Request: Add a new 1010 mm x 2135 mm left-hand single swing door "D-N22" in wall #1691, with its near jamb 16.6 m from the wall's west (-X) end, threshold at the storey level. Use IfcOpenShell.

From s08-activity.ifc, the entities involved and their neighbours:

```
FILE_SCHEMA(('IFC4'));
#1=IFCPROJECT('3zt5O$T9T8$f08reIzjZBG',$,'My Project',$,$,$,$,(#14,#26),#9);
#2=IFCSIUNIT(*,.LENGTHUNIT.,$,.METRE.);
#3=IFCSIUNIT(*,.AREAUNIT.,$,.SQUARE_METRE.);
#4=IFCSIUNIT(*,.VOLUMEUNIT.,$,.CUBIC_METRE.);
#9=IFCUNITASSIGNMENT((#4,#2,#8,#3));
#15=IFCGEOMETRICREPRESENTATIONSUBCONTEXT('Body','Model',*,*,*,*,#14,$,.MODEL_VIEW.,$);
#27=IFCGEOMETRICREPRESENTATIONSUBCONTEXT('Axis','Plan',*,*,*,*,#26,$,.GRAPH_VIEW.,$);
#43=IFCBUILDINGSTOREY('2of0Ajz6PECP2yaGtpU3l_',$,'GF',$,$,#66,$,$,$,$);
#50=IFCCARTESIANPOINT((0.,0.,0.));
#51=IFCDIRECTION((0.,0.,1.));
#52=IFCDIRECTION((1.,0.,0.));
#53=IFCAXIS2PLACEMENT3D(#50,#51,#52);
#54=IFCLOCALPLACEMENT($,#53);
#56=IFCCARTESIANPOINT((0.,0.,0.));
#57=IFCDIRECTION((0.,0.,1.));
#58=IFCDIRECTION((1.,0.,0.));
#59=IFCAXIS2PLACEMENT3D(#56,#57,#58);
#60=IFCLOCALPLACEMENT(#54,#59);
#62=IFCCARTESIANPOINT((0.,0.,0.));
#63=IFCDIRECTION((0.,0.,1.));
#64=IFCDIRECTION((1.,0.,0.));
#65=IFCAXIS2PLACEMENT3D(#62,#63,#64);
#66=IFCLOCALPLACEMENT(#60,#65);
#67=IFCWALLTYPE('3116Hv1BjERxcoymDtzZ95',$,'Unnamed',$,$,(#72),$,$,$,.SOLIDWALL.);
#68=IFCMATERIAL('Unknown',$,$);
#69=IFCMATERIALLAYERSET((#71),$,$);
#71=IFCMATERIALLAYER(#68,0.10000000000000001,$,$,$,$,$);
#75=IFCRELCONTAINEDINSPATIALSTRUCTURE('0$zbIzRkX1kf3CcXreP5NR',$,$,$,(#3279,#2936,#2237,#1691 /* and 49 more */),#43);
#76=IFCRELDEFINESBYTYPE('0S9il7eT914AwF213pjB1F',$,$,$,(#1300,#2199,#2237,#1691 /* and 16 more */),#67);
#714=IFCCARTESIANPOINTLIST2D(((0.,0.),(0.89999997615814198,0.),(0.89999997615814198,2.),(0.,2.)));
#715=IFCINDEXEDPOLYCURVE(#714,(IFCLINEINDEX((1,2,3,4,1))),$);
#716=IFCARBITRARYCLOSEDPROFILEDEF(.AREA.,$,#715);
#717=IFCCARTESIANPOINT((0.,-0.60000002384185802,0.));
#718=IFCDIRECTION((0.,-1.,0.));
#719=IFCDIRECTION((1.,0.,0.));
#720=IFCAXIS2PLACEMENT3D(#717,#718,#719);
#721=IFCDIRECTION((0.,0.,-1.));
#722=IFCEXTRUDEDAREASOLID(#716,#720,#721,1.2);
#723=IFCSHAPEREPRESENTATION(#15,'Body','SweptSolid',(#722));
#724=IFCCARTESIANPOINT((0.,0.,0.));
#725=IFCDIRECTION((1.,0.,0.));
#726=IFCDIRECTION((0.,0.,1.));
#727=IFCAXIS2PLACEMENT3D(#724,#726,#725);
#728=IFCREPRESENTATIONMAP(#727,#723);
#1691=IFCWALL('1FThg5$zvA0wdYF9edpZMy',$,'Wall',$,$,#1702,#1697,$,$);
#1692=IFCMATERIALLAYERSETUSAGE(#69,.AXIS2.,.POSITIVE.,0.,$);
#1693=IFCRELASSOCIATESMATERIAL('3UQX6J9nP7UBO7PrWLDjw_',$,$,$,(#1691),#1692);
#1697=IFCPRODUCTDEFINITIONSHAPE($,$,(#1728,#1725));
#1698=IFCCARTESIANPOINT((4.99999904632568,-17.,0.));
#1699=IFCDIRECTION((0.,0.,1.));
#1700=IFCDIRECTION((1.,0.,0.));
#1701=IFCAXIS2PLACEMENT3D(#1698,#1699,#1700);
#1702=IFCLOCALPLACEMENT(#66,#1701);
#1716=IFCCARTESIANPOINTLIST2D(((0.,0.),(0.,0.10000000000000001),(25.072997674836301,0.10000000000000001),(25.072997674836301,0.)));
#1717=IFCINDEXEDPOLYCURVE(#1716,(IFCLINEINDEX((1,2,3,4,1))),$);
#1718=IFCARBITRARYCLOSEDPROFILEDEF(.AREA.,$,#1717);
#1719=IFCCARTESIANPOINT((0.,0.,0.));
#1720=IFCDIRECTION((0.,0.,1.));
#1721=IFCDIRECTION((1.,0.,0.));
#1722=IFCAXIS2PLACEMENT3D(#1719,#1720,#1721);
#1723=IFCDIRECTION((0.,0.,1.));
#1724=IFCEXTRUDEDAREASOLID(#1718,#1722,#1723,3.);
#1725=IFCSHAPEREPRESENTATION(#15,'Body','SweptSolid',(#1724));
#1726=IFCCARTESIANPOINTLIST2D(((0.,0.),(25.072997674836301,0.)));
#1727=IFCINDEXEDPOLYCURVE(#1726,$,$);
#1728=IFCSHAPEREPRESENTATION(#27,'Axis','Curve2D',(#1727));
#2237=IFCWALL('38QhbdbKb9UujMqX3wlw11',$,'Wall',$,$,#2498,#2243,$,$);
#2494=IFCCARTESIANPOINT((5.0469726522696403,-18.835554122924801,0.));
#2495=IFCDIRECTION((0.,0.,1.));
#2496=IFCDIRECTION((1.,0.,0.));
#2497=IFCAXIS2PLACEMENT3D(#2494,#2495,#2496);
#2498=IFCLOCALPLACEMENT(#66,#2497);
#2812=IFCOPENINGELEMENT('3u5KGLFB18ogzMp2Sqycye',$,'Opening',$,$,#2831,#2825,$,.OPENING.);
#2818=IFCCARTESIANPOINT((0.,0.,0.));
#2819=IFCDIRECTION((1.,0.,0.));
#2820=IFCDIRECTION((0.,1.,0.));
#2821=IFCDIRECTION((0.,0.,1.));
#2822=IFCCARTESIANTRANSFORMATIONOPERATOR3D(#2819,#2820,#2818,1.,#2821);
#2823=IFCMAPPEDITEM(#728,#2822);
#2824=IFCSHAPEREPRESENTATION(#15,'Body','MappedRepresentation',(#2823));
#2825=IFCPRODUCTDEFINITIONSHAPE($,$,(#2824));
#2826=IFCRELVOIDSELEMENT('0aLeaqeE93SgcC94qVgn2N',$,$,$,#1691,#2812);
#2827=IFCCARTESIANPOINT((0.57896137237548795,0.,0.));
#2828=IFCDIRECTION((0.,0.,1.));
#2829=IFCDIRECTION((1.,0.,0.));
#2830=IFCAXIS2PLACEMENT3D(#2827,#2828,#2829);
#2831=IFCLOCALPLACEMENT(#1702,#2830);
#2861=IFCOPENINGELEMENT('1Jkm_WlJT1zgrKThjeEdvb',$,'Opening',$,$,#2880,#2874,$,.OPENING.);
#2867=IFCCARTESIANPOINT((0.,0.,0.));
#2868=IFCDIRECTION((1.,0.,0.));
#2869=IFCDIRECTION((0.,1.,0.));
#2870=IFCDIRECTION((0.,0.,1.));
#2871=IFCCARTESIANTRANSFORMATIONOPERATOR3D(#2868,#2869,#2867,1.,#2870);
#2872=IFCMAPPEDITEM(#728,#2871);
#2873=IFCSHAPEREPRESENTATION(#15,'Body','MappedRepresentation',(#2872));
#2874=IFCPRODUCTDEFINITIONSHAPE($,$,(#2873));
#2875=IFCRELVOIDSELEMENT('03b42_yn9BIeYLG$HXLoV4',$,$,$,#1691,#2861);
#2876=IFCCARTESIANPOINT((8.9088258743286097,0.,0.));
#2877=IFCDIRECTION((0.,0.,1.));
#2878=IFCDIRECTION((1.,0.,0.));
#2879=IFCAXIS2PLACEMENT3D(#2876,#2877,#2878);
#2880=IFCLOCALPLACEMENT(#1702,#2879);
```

```python
import numpy as np
import ifcopenshell
import ifcopenshell.api.feature
import ifcopenshell.api.geometry
import ifcopenshell.api.root
import ifcopenshell.api.spatial
import ifcopenshell.geom
import ifcopenshell.util.element
import ifcopenshell.util.placement
import ifcopenshell.util.representation
import ifcopenshell.util.shape
import ifcopenshell.util.unit

model = ifcopenshell.open("s08-activity.ifc")
unit_scale = ifcopenshell.util.unit.calculate_unit_scale(model)
settings = ifcopenshell.geom.settings()


def volume(element):
    """Net volume in cubic metres, openings subtracted."""
    shape = ifcopenshell.geom.create_shape(settings, element)
    return ifcopenshell.util.shape.get_volume(shape.geometry)


wall = model.by_guid("1FThg5$zvA0wdYF9edpZMy")
storey = ifcopenshell.util.element.get_container(wall, ifc_class="IfcBuildingStorey")
context = ifcopenshell.util.representation.get_context(model, "Model", "Body", "MODEL_VIEW")
before = volume(wall)

width, height, from_end, sill = 1.01, 2.135, 16.6, 0.0  # metres

# The wall runs along its own X axis, and the end named is its -X end.
wall_shape = ifcopenshell.geom.create_shape(settings, wall)
x, y, z = ifcopenshell.util.shape.get_vertices(wall_shape.geometry).T
start = x.min() + from_end
face, thickness = float(y.min()), float(y.max() - y.min())
wall_matrix = ifcopenshell.util.placement.get_local_placement(wall.ObjectPlacement)
level = ifcopenshell.util.placement.get_local_placement(storey.ObjectPlacement)[2, 3]


def in_wall(x, y):
    """Placement at x, y metres in the wall's axes, at sill height."""
    matrix = wall_matrix.copy()
    matrix[:, 3] = wall_matrix @ np.array([x / unit_scale, y / unit_scale, 0.0, 1.0])
    matrix[2, 3] = level + sill / unit_scale
    return matrix


# Opening: a box that overshoots both wall faces by 50 mm.
opening = ifcopenshell.api.root.create_entity(model, ifc_class="IfcOpeningElement", predefined_type="OPENING")
box = ifcopenshell.api.geometry.add_wall_representation(
    model, context=context, length=width, height=height, thickness=thickness + 0.1
)
ifcopenshell.api.geometry.assign_representation(model, product=opening, representation=box)
ifcopenshell.api.geometry.edit_object_placement(model, product=opening, matrix=in_wall(start, face - 0.05), is_si=False)
ifcopenshell.api.feature.add_feature(model, feature=opening, element=wall)

door = ifcopenshell.api.root.create_entity(model, ifc_class="IfcDoor", name="D-N22", predefined_type="DOOR")
door.OverallWidth, door.OverallHeight = width / unit_scale, height / unit_scale
door.OperationType = "SINGLE_SWING_LEFT"
body = ifcopenshell.api.geometry.add_door_representation(
    model,
    context=context,
    overall_width=door.OverallWidth,
    overall_height=door.OverallHeight,
    operation_type="SINGLE_SWING_LEFT",
    lining_properties={"LiningDepth": thickness / unit_scale, "ThresholdDepth": thickness / unit_scale},
)
ifcopenshell.api.geometry.assign_representation(model, product=door, representation=body)
ifcopenshell.api.spatial.assign_container(model, products=[door], relating_structure=storey)
ifcopenshell.api.feature.add_filling(model, opening=opening, element=door)

# The lining spans the wall, so the door starts at the wall face.
ifcopenshell.api.geometry.edit_object_placement(model, product=door, matrix=in_wall(start, face), is_si=False)

after = volume(wall)

print(f"wall volume {before:.3f} -> {after:.3f} m3")

model.write("s08-activity-out.ifc")
```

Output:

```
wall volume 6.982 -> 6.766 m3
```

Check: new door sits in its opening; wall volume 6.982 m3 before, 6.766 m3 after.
